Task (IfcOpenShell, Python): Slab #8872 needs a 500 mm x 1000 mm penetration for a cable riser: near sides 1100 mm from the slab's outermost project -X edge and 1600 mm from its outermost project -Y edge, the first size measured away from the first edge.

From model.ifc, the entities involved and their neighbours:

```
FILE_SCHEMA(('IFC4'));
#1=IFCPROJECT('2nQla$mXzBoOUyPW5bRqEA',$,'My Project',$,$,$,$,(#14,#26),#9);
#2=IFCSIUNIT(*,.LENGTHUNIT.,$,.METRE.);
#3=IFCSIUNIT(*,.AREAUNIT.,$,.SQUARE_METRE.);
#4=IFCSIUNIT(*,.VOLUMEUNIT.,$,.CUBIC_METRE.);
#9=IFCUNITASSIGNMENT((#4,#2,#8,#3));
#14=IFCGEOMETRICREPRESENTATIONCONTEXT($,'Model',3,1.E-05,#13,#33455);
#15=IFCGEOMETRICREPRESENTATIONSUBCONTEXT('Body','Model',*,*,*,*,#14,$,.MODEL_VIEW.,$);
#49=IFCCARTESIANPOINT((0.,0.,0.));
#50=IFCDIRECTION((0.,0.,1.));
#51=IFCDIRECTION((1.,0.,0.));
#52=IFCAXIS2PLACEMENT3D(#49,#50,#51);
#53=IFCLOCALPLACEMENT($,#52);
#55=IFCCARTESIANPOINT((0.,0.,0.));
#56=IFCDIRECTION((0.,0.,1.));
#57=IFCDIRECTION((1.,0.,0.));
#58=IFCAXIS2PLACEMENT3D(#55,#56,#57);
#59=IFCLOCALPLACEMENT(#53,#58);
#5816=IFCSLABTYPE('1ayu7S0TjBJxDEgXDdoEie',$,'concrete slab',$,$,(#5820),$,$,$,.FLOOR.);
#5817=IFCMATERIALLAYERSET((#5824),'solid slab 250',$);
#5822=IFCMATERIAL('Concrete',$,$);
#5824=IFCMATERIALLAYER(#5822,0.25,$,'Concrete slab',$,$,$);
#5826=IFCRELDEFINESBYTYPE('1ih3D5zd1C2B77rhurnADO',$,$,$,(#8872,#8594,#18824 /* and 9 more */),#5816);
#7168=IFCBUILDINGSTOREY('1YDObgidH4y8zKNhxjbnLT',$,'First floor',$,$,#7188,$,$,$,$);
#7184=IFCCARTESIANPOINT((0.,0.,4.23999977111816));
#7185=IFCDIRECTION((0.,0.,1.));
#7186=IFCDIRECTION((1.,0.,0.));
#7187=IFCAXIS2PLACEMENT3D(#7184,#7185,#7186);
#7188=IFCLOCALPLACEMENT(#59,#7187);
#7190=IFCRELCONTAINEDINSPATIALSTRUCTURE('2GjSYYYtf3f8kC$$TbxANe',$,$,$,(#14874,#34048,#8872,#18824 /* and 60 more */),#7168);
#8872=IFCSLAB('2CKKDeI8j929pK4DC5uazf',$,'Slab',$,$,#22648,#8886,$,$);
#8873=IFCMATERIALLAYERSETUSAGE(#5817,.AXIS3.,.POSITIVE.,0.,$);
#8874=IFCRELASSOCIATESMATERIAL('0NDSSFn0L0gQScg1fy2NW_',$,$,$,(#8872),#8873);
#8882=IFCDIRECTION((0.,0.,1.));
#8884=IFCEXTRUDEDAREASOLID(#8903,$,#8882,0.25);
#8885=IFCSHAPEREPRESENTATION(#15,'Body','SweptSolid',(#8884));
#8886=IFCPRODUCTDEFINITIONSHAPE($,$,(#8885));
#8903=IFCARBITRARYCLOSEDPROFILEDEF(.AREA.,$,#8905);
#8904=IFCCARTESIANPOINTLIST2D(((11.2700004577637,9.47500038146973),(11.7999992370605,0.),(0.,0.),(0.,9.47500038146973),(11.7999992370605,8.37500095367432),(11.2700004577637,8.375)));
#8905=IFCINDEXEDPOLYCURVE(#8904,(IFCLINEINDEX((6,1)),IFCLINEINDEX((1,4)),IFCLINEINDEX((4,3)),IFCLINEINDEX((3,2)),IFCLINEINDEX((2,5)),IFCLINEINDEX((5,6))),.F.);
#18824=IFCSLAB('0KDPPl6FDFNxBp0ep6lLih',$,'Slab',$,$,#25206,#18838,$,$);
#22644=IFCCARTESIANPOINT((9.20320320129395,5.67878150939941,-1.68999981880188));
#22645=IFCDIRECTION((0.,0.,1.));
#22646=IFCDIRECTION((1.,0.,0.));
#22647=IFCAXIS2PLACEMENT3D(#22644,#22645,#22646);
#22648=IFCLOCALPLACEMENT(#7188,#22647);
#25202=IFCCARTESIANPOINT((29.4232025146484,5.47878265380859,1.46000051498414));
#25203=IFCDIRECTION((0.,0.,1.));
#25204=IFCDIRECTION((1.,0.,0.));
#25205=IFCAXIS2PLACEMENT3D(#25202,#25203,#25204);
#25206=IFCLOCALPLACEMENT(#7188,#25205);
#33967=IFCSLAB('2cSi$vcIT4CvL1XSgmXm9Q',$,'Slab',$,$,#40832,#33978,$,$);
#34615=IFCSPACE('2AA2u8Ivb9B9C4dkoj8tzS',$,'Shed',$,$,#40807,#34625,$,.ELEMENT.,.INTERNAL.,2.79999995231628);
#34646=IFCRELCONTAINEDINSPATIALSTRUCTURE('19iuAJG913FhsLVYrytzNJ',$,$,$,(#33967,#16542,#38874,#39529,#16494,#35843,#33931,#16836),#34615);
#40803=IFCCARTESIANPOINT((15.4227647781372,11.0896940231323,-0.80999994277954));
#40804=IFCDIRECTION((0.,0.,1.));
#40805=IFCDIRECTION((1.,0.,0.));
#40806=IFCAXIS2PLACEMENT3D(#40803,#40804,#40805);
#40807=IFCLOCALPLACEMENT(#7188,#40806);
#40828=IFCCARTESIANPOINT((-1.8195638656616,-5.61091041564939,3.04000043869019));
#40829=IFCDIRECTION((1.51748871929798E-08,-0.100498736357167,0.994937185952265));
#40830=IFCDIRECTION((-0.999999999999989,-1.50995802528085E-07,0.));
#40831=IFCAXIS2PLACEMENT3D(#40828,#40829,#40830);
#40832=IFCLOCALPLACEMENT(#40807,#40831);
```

```python
import numpy as np
import ifcopenshell
import ifcopenshell.api.feature
import ifcopenshell.api.geometry
import ifcopenshell.api.root
import ifcopenshell.geom
import ifcopenshell.util.placement
import ifcopenshell.util.representation
import ifcopenshell.util.shape
import ifcopenshell.util.unit

model = ifcopenshell.open("model.ifc")
unit_scale = ifcopenshell.util.unit.calculate_unit_scale(model)
settings = ifcopenshell.geom.settings()


def volume(element):
    """Net volume in cubic metres, openings subtracted."""
    shape = ifcopenshell.geom.create_shape(settings, element)
    return ifcopenshell.util.shape.get_volume(shape.geometry)


slab = model.by_guid("2CKKDeI8j929pK4DC5uazf")
before = volume(slab)

# Extent in the slab's own axes, in metres. The edges named are its -X and -Y sides.
slab_shape = ifcopenshell.geom.create_shape(settings, slab)
vertices = ifcopenshell.util.shape.get_vertices(slab_shape.geometry)
x_min, y_min, bottom = vertices.min(axis=0)
top = vertices[:, 2].max()

opening = ifcopenshell.api.root.create_entity(model, ifc_class="IfcOpeningElement", name="Cable riser opening", predefined_type="OPENING")
context = ifcopenshell.util.representation.get_context(model, "Model", "Body", "MODEL_VIEW")
width, depth = 0.5, 1
outline = [(0.0, 0.0), (width, 0.0), (width, depth), (0.0, depth), (0.0, 0.0)]
# Overshoot both faces by 50 mm so the cut is clean.
shape = ifcopenshell.api.geometry.add_slab_representation(
    model, context=context, depth=top - bottom + 0.1, polyline=outline
)
ifcopenshell.api.geometry.assign_representation(model, product=opening, representation=shape)

matrix = ifcopenshell.util.placement.get_local_placement(slab.ObjectPlacement)
matrix[:, 3] = matrix @ np.append(np.array([x_min + 1.1, y_min + 1.6, bottom - 0.05]) / unit_scale, 1.0)
ifcopenshell.api.geometry.edit_object_placement(model, product=opening, matrix=matrix, is_si=False)
ifcopenshell.api.feature.add_feature(model, feature=opening, element=slab)

after = volume(slab)

print(f"slab volume {before:.3f} -> {after:.3f} m3")

model.write("model_v2.ifc")
```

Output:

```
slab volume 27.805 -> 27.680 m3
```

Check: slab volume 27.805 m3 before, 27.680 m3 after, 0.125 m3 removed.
